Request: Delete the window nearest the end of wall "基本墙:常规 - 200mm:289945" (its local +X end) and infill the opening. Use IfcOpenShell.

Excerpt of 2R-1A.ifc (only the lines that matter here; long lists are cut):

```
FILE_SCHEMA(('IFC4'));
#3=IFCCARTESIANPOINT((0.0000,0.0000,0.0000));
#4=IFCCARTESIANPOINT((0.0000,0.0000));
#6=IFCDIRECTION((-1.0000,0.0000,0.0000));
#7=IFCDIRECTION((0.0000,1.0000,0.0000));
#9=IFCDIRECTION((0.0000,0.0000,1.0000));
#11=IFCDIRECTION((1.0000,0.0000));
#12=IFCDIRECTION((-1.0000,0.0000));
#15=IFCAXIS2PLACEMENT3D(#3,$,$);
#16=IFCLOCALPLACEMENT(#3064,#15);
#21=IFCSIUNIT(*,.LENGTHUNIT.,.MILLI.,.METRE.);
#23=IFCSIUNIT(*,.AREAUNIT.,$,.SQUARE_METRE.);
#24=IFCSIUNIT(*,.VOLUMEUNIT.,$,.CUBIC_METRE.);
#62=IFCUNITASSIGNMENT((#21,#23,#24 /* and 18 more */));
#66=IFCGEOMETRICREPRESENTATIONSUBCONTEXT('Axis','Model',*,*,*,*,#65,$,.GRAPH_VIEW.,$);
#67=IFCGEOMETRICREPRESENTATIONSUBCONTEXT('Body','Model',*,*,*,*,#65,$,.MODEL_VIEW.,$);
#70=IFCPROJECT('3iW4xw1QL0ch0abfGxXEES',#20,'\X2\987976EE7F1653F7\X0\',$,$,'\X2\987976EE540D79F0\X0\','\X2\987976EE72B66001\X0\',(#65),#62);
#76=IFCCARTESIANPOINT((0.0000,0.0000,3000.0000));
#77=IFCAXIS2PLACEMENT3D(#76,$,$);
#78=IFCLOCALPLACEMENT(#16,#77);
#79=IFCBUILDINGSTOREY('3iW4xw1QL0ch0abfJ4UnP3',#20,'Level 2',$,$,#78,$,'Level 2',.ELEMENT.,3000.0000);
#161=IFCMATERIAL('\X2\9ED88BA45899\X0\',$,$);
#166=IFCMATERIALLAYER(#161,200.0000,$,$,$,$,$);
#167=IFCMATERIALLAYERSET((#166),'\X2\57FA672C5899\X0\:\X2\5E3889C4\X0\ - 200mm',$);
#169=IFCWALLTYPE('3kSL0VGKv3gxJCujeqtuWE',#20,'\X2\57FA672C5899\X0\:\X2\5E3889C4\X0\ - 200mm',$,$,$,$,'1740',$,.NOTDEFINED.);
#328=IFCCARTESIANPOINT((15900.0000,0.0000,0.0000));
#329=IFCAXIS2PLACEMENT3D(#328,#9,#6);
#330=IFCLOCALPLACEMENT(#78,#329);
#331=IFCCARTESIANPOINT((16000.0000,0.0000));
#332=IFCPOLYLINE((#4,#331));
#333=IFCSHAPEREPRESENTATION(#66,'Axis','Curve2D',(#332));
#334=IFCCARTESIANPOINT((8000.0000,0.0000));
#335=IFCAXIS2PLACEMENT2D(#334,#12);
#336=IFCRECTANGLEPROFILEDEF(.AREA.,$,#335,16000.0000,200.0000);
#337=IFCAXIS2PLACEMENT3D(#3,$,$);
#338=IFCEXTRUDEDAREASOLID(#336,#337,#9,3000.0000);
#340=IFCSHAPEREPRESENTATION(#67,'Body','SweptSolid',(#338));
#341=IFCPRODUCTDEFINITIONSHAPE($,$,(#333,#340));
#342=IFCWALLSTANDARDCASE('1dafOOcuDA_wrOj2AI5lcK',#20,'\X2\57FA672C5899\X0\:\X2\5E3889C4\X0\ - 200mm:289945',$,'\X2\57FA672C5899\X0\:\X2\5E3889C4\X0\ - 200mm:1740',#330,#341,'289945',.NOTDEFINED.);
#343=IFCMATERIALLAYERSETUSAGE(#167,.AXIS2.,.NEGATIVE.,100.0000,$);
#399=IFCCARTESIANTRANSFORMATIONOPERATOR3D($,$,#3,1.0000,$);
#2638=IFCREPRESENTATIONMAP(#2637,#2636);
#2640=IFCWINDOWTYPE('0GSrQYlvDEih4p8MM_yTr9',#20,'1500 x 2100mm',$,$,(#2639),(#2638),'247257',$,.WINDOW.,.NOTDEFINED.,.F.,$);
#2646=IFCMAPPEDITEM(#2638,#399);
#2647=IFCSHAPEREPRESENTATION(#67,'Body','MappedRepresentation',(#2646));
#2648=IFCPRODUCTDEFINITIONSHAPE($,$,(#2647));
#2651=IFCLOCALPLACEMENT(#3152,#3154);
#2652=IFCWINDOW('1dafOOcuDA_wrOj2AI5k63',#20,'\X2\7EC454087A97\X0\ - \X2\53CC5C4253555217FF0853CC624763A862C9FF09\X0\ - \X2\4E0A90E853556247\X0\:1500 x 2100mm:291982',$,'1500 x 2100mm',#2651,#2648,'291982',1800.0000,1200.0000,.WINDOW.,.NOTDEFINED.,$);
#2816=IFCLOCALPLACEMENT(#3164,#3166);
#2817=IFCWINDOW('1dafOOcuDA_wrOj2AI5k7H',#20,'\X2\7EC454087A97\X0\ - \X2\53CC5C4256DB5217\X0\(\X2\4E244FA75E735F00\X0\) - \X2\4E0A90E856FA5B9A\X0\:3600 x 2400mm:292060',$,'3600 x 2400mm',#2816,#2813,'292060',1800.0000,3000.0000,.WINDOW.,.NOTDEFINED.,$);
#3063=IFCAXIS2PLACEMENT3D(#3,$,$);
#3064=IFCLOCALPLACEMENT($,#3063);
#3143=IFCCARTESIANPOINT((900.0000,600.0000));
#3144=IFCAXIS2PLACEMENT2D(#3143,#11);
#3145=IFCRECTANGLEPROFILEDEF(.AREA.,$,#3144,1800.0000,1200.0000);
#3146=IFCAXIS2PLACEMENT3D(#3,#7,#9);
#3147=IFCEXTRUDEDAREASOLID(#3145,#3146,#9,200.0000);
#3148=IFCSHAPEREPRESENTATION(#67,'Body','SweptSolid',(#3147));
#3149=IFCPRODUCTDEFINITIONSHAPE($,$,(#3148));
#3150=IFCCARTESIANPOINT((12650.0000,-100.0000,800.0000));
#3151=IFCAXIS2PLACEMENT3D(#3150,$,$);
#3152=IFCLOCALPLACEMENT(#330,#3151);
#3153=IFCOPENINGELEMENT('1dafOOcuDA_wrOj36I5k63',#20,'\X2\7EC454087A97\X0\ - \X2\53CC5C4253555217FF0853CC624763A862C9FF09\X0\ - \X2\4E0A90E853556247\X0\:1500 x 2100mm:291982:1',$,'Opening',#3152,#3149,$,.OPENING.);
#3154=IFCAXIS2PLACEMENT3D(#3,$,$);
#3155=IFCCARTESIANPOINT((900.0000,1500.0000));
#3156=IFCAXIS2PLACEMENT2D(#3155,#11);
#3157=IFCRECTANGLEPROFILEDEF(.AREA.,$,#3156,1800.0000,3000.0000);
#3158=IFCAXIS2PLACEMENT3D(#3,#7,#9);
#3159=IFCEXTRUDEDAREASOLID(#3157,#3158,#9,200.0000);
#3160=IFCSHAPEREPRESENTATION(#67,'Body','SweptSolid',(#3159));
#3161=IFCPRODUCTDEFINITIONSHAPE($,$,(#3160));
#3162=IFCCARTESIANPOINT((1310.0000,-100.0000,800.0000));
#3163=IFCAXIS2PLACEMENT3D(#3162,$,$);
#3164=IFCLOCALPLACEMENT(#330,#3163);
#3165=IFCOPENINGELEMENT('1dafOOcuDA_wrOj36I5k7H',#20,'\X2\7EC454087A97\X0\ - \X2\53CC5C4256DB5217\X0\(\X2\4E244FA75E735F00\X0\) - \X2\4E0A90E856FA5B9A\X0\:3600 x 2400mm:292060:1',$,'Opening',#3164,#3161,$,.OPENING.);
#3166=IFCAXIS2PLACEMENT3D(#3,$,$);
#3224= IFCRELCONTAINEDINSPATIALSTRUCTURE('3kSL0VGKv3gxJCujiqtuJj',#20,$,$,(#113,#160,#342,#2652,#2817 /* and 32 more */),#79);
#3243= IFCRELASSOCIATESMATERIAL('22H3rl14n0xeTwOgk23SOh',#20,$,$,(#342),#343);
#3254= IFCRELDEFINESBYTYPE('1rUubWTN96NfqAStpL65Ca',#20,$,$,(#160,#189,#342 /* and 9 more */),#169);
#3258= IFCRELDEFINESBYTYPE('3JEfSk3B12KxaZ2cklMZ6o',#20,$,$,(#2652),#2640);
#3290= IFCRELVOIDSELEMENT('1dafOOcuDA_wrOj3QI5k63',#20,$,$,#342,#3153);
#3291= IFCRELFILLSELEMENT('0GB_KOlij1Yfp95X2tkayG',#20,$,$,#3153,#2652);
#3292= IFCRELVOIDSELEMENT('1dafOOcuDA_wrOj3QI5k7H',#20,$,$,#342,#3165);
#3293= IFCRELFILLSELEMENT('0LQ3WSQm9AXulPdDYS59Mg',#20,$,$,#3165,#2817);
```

```python
import ifcopenshell
import ifcopenshell.api.feature
import ifcopenshell.api.root
import ifcopenshell.geom
import ifcopenshell.util.shape

model = ifcopenshell.open("2R-1A.ifc")
settings = ifcopenshell.geom.settings()


def volume(element):
    """Net volume in cubic metres, openings subtracted."""
    shape = ifcopenshell.geom.create_shape(settings, element)
    return ifcopenshell.util.shape.get_volume(shape.geometry)


window = model.by_guid("1dafOOcuDA_wrOj2AI5k63")
opening = window.FillsVoids[0].RelatingOpeningElement
wall = opening.VoidsElements[0].RelatingBuildingElement
before = volume(wall)

ifcopenshell.api.root.remove_product(model, product=window)
ifcopenshell.api.feature.remove_feature(model, feature=opening)

after = volume(wall)

print(f"wall volume {before:.3f} -> {after:.3f} m3")

model.write("2R-1A_v2.ifc")
```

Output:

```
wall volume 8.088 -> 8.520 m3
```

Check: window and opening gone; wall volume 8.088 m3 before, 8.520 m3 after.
